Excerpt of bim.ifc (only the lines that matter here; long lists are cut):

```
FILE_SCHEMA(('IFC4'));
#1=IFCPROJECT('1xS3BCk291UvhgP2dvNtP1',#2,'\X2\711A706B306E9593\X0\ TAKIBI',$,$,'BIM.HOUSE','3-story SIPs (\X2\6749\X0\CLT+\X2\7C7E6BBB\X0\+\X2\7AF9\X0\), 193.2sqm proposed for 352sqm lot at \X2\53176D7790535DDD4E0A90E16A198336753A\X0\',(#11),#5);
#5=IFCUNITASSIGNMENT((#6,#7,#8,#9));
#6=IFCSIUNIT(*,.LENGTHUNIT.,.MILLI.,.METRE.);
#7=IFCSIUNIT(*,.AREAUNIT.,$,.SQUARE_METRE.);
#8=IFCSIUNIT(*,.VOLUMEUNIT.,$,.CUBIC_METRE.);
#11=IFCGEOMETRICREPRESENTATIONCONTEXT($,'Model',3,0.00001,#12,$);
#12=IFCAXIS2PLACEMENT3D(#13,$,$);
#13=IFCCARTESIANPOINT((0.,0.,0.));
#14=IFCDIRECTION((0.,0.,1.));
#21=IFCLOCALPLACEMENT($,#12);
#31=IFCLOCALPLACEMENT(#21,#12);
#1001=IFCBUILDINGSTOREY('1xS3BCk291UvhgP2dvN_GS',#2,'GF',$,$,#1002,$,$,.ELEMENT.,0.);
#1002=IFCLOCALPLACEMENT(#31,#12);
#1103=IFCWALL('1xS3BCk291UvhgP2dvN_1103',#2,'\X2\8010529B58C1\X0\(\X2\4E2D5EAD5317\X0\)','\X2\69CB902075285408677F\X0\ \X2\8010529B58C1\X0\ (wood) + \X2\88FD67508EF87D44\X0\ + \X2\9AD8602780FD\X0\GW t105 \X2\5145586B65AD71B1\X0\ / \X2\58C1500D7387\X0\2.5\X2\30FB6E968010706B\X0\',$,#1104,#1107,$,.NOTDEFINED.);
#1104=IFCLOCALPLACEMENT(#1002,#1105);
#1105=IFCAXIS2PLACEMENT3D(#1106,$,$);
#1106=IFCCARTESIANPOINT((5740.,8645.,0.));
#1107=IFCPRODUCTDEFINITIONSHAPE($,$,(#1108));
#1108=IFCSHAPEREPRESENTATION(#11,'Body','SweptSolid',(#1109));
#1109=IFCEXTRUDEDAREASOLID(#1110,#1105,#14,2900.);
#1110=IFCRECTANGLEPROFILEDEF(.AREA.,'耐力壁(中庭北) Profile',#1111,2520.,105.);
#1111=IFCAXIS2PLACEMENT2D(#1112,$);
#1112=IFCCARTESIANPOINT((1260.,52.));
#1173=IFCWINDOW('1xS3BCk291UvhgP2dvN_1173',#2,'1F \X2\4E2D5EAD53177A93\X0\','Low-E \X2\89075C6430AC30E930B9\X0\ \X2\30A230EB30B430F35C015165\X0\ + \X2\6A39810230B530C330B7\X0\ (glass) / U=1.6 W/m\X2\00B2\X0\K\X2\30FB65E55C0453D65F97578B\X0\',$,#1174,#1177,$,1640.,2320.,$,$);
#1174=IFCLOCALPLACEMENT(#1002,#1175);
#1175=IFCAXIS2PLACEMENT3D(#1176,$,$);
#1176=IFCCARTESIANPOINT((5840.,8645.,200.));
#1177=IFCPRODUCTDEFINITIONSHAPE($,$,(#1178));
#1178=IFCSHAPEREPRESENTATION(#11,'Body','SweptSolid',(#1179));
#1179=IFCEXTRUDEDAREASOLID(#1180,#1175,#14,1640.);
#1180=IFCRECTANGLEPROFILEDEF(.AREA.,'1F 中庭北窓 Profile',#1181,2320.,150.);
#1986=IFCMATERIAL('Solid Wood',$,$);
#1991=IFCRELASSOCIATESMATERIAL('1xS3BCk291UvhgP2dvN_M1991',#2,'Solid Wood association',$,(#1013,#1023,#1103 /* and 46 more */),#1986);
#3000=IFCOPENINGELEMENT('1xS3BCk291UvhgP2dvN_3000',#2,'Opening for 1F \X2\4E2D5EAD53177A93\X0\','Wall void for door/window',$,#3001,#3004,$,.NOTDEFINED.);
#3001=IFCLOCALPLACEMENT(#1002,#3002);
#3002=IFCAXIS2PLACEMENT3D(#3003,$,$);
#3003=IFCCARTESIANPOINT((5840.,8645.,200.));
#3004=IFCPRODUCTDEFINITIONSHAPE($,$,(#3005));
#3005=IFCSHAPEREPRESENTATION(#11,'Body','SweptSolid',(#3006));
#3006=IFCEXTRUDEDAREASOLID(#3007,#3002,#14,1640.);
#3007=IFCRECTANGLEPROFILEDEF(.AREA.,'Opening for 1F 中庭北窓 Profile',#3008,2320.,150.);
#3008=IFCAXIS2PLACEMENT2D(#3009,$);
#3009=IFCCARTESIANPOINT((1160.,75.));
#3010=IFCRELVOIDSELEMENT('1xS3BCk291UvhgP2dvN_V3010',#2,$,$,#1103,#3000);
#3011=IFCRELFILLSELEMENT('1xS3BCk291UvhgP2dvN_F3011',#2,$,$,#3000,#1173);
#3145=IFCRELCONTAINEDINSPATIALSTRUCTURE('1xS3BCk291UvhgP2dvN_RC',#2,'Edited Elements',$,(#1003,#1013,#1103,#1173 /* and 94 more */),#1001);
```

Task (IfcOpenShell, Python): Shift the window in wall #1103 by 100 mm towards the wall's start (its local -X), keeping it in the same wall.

```python
import ifcopenshell
import ifcopenshell.api.geometry
import ifcopenshell.util.placement
import ifcopenshell.util.unit

model = ifcopenshell.open("bim.ifc")
unit_scale = ifcopenshell.util.unit.calculate_unit_scale(model)

window = model.by_id(1173)
opening = window.FillsVoids[0].RelatingOpeningElement
wall = opening.VoidsElements[0].RelatingBuildingElement

wall_matrix = ifcopenshell.util.placement.get_local_placement(wall.ObjectPlacement)
shift = wall_matrix[:3, 0] * -0.1 / unit_scale
before = ifcopenshell.util.placement.get_local_placement(window.ObjectPlacement)[:3, 3].copy()

# The window is not placed relative to its opening, so move both.
for product in (opening, window):
    matrix = ifcopenshell.util.placement.get_local_placement(product.ObjectPlacement)
    matrix[:3, 3] += shift
    ifcopenshell.api.geometry.edit_object_placement(model, product=product, matrix=matrix, is_si=False)

after = ifcopenshell.util.placement.get_local_placement(window.ObjectPlacement)[:3, 3]
print("window moved by", (after - before).round(3) + 0.0)

model.write("bim-out.ifc")
```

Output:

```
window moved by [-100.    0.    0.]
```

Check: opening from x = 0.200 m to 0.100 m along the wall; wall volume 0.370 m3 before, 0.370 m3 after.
